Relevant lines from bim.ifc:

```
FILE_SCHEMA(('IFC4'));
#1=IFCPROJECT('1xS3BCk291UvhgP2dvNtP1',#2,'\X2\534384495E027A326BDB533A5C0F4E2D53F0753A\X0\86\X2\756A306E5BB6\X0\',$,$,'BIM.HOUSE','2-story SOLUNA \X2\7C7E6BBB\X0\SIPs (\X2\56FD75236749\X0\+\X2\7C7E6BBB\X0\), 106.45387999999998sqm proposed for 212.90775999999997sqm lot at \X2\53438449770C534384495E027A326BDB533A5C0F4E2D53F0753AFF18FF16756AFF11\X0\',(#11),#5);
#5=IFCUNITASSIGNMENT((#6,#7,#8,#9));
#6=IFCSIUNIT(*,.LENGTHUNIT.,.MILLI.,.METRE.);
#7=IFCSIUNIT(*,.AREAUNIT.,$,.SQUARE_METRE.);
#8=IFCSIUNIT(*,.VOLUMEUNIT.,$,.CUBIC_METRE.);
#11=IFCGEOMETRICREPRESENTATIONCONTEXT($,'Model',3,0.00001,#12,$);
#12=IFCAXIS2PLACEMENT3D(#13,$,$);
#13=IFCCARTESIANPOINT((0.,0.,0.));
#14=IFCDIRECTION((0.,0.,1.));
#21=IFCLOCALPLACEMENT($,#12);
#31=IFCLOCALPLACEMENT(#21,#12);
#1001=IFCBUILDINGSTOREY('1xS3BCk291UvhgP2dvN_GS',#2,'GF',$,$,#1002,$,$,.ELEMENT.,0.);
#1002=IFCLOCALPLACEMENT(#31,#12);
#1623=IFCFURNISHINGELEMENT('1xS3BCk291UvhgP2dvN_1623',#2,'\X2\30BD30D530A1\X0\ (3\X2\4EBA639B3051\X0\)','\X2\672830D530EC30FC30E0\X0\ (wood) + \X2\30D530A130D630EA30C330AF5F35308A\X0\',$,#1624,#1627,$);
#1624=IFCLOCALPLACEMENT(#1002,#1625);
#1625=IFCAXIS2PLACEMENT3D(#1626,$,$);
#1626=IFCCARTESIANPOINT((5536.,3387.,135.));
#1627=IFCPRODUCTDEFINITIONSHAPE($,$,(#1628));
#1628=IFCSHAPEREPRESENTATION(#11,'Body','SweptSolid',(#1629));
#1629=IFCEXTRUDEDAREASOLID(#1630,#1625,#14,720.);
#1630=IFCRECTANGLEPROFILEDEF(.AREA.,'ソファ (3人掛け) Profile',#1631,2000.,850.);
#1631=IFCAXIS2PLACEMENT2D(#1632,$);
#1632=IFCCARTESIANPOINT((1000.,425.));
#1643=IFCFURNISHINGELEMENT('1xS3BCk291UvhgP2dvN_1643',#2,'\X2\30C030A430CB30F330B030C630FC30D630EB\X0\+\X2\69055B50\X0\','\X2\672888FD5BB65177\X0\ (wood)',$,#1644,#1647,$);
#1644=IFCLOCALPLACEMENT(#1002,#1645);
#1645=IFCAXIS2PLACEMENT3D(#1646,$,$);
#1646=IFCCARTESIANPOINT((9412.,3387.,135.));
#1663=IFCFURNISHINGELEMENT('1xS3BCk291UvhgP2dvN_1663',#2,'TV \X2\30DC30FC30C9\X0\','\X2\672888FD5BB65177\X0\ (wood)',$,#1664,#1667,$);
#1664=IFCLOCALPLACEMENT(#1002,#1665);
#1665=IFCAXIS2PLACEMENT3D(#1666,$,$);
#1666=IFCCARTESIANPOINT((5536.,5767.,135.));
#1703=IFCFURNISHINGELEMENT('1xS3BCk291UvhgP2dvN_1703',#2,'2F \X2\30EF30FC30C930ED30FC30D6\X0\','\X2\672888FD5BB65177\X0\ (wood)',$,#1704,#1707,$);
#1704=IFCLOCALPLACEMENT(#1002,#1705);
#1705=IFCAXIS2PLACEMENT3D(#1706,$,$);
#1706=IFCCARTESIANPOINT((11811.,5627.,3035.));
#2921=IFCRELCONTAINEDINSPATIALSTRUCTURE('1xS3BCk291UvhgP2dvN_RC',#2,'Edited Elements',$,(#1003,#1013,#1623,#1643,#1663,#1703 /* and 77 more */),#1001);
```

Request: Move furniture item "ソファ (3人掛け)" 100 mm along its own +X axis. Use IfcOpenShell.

```python
import ifcopenshell
import ifcopenshell.api.geometry
import ifcopenshell.util.placement
import ifcopenshell.util.unit

model = ifcopenshell.open("bim.ifc")
unit_scale = ifcopenshell.util.unit.calculate_unit_scale(model)

item = model.by_guid("1xS3BCk291UvhgP2dvN_1623")
matrix = ifcopenshell.util.placement.get_local_placement(item.ObjectPlacement)
matrix[:3, 3] += matrix[:3, 0] * 0.1 / unit_scale
ifcopenshell.api.geometry.edit_object_placement(model, product=item, matrix=matrix, is_si=False)

print(ifcopenshell.util.placement.get_local_placement(item.ObjectPlacement).round(3) + 0.0)

model.write("bim_updated.ifc")
```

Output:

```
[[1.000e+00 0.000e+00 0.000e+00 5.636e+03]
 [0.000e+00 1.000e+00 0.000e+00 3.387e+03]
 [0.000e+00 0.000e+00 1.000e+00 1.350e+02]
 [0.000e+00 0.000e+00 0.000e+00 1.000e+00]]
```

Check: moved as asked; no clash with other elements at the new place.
